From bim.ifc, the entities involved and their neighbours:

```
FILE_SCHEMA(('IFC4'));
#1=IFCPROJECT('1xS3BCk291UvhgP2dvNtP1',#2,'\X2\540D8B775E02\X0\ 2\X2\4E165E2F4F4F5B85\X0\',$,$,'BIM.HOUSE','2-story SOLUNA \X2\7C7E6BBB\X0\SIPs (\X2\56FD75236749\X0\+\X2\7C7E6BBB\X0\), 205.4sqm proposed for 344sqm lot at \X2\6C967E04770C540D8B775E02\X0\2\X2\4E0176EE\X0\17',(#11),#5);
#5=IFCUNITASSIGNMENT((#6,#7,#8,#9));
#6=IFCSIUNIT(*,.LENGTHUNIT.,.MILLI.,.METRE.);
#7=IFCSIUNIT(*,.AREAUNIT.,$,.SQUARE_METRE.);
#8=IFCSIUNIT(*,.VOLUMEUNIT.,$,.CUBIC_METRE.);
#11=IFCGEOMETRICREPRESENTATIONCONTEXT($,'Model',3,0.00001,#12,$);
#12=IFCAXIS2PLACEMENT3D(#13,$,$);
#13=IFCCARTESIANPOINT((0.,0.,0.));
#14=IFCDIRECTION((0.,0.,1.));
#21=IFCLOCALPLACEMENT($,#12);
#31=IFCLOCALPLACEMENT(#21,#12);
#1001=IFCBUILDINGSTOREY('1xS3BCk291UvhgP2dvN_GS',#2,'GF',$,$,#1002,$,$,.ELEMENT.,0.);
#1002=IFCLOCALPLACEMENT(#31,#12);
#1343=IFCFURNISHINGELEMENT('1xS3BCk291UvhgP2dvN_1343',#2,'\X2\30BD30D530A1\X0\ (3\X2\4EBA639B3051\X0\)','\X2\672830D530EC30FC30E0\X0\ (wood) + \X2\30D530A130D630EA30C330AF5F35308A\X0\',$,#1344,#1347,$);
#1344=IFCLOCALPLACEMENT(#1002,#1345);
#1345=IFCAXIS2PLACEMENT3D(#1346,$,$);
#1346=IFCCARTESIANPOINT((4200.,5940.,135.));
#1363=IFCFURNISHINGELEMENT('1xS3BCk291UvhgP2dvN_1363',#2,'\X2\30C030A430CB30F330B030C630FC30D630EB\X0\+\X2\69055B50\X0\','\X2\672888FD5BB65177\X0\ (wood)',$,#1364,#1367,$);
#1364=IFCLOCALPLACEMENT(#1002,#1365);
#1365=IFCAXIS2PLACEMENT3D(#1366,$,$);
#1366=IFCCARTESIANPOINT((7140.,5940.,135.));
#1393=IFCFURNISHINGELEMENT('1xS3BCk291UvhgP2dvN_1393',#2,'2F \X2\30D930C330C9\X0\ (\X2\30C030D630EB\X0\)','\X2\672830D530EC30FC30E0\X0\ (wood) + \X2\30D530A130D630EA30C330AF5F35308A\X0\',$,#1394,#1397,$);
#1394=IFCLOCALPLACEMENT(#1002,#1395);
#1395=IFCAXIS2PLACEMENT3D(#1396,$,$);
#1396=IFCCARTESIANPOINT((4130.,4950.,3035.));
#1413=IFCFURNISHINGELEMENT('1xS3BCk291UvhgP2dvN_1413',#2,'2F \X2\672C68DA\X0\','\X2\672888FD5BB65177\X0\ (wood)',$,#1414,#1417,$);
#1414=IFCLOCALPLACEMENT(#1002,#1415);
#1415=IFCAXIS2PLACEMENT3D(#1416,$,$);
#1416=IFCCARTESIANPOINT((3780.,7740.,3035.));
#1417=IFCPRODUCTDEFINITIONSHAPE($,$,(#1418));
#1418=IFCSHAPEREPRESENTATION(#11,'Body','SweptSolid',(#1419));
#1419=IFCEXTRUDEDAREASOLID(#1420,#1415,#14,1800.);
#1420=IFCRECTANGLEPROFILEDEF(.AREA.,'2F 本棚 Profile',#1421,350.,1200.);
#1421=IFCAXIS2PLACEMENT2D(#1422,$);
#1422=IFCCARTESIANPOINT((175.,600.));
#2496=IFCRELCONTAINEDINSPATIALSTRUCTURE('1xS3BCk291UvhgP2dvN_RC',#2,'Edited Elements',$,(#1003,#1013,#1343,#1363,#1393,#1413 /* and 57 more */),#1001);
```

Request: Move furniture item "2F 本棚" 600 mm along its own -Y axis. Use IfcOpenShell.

```python
import ifcopenshell
import ifcopenshell.api.geometry
import ifcopenshell.util.placement
import ifcopenshell.util.unit

model = ifcopenshell.open("bim.ifc")
unit_scale = ifcopenshell.util.unit.calculate_unit_scale(model)

item = model.by_guid("1xS3BCk291UvhgP2dvN_1413")
matrix = ifcopenshell.util.placement.get_local_placement(item.ObjectPlacement)
matrix[:3, 3] -= matrix[:3, 1] * 0.6 / unit_scale
ifcopenshell.api.geometry.edit_object_placement(model, product=item, matrix=matrix, is_si=False)

print(ifcopenshell.util.placement.get_local_placement(item.ObjectPlacement).round(3) + 0.0)

model.write("bim_edited.ifc")
```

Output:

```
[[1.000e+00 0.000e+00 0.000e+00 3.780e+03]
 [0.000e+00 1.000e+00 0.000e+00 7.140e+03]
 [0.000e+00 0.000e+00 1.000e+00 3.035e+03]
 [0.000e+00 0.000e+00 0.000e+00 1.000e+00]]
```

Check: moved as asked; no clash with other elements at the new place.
